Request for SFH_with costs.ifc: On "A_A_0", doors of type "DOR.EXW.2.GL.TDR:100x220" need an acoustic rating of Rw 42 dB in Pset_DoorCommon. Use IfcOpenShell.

First a look at what the model holds.

```python
import ifcopenshell
import ifcopenshell.util.element

model = ifcopenshell.open("SFH_with costs.ifc")
print(model.schema)
storey = next(s for s in model.by_type("IfcBuildingStorey") if s.Name == "A_A_0")
doors = [e for e in ifcopenshell.util.element.get_decomposition(storey) if e.is_a("IfcDoor")]
seen = {}
for e in doors:
    element_type = ifcopenshell.util.element.get_type(e)
    key = (element_type.Name if element_type != e and element_type else None, ifcopenshell.util.element.get_pset(e, "Pset_DoorCommon", "AcousticRating"))
    seen[key] = seen.get(key, 0) + 1
for (name, value), count in sorted(seen.items(), key=str):
    print(count, "x", name, "|", value)
```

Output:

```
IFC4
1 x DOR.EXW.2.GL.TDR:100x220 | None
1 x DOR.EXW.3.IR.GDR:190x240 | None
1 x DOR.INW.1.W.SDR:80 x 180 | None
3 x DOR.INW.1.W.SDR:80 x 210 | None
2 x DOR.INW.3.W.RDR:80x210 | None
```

```python
import ifcopenshell
import ifcopenshell.api.pset
import ifcopenshell.util.element

model = ifcopenshell.open("SFH_with costs.ifc")

storey = next(s for s in model.by_type("IfcBuildingStorey") if s.Name == "A_A_0")
doors = [e for e in ifcopenshell.util.element.get_decomposition(storey) if e.is_a("IfcDoor")]

count = 0
for e in doors:
    element_type = ifcopenshell.util.element.get_type(e)
    if element_type in (None, e) or element_type.Name != "DOR.EXW.2.GL.TDR:100x220":
        continue
    # add_pset returns the element's existing set when there is one.
    pset = ifcopenshell.api.pset.add_pset(model, product=e, name="Pset_DoorCommon")
    ifcopenshell.api.pset.edit_pset(model, pset=pset, properties={"AcousticRating": "Rw 42 dB"})
    count += 1

print(count, "doors updated")

model.write("SFH_with costs_rev.ifc")
```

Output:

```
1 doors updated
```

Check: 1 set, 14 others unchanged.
